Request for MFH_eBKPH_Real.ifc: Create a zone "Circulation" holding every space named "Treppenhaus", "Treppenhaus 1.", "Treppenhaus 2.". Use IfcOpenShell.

First a look at what the model holds.

```python
import ifcopenshell

model = ifcopenshell.open("MFH_eBKPH_Real.ifc")
print(model.schema)
seen = {}
for space in model.by_type("IfcSpace"):
    seen[space.LongName] = seen.get(space.LongName, 0) + 1
for name, count in sorted(seen.items(), key=str):
    print(count, "x", name)
print("zones:", [z.Name for z in model.by_type("IfcZone")][:20])
```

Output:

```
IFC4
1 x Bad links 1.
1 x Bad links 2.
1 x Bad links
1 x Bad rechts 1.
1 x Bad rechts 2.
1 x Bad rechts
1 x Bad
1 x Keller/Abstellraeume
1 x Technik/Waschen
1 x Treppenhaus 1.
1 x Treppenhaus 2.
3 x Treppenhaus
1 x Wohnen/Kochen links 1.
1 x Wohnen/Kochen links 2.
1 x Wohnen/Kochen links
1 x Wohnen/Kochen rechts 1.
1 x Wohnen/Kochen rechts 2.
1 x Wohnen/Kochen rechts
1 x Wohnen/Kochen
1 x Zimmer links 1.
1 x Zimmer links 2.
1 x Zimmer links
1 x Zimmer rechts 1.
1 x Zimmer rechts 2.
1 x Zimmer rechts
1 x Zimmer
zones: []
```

```python
import ifcopenshell
import ifcopenshell.api.group
import ifcopenshell.api.root

model = ifcopenshell.open("MFH_eBKPH_Real.ifc")

names = {"Treppenhaus", "Treppenhaus 1.", "Treppenhaus 2."}
spaces = [s for s in model.by_type("IfcSpace") if s.LongName in names]

zone = ifcopenshell.api.root.create_entity(model, ifc_class="IfcZone", name="Circulation")
ifcopenshell.api.group.assign_group(model, products=spaces, group=zone)
print(len(spaces), "spaces in", zone.Name)

model.write("MFH_eBKPH_Real_rev.ifc")
```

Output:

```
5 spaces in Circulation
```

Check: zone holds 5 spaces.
